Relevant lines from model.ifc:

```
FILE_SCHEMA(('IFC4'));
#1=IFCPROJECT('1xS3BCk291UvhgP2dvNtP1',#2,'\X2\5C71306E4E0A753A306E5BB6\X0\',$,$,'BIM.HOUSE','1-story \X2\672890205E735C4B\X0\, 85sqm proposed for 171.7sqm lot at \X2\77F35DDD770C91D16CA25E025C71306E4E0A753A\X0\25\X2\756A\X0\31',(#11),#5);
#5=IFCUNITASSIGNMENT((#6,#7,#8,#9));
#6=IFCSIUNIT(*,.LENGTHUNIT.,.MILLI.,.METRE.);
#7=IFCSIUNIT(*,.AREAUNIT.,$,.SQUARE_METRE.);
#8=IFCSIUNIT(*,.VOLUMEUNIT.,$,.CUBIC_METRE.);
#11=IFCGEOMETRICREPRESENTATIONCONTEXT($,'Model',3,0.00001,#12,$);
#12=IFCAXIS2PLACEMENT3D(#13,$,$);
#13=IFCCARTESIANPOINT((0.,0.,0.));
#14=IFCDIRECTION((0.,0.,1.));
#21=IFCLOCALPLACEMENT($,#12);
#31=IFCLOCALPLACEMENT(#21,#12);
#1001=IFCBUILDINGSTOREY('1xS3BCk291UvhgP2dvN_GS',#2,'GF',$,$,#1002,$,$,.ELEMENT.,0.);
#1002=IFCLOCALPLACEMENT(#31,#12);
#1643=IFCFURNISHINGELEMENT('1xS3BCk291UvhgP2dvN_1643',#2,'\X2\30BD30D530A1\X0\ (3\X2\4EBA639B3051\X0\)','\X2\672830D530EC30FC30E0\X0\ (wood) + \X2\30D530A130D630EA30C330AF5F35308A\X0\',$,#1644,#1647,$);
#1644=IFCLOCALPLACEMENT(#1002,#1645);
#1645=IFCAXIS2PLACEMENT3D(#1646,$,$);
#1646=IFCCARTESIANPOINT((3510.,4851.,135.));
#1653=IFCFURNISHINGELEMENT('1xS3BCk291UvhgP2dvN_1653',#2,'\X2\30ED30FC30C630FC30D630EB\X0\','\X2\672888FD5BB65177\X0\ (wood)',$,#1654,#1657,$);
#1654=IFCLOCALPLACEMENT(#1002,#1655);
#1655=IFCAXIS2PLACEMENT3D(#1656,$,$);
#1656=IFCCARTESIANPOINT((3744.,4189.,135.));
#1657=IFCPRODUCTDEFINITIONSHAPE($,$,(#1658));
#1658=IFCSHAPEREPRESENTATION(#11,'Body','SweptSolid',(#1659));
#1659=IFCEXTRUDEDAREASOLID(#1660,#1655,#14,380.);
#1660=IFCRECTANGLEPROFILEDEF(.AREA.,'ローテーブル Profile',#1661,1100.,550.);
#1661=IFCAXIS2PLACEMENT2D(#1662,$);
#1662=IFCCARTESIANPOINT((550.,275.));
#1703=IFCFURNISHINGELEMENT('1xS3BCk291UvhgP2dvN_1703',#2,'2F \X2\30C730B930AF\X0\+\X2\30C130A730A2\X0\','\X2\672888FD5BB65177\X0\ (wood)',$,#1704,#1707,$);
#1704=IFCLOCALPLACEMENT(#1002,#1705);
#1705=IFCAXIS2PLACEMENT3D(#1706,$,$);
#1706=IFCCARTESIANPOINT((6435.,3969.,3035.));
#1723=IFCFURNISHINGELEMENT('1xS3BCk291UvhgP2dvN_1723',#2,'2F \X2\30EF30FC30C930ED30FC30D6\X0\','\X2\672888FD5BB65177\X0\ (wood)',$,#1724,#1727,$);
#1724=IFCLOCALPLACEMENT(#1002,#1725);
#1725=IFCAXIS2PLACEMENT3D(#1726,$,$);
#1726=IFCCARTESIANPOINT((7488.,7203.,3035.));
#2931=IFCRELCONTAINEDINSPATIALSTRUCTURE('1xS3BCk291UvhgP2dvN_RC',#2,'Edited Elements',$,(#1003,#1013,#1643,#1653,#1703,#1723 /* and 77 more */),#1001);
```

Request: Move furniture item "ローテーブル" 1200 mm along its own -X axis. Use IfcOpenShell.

```python
import ifcopenshell
import ifcopenshell.api.geometry
import ifcopenshell.util.placement

model = ifcopenshell.open("model.ifc")

item = model.by_guid("1xS3BCk291UvhgP2dvN_1653")
matrix = ifcopenshell.util.placement.get_local_placement(item.ObjectPlacement)
matrix[:3, 3] -= matrix[:3, 0] * 1200.0
ifcopenshell.api.geometry.edit_object_placement(model, product=item, matrix=matrix, is_si=False)

print(ifcopenshell.util.placement.get_local_placement(item.ObjectPlacement).round(3) + 0.0)

model.write("model_v2.ifc")
```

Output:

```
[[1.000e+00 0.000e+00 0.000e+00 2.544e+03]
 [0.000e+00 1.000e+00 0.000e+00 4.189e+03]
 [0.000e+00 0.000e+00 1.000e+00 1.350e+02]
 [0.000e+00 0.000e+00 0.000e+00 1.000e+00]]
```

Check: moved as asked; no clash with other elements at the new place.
